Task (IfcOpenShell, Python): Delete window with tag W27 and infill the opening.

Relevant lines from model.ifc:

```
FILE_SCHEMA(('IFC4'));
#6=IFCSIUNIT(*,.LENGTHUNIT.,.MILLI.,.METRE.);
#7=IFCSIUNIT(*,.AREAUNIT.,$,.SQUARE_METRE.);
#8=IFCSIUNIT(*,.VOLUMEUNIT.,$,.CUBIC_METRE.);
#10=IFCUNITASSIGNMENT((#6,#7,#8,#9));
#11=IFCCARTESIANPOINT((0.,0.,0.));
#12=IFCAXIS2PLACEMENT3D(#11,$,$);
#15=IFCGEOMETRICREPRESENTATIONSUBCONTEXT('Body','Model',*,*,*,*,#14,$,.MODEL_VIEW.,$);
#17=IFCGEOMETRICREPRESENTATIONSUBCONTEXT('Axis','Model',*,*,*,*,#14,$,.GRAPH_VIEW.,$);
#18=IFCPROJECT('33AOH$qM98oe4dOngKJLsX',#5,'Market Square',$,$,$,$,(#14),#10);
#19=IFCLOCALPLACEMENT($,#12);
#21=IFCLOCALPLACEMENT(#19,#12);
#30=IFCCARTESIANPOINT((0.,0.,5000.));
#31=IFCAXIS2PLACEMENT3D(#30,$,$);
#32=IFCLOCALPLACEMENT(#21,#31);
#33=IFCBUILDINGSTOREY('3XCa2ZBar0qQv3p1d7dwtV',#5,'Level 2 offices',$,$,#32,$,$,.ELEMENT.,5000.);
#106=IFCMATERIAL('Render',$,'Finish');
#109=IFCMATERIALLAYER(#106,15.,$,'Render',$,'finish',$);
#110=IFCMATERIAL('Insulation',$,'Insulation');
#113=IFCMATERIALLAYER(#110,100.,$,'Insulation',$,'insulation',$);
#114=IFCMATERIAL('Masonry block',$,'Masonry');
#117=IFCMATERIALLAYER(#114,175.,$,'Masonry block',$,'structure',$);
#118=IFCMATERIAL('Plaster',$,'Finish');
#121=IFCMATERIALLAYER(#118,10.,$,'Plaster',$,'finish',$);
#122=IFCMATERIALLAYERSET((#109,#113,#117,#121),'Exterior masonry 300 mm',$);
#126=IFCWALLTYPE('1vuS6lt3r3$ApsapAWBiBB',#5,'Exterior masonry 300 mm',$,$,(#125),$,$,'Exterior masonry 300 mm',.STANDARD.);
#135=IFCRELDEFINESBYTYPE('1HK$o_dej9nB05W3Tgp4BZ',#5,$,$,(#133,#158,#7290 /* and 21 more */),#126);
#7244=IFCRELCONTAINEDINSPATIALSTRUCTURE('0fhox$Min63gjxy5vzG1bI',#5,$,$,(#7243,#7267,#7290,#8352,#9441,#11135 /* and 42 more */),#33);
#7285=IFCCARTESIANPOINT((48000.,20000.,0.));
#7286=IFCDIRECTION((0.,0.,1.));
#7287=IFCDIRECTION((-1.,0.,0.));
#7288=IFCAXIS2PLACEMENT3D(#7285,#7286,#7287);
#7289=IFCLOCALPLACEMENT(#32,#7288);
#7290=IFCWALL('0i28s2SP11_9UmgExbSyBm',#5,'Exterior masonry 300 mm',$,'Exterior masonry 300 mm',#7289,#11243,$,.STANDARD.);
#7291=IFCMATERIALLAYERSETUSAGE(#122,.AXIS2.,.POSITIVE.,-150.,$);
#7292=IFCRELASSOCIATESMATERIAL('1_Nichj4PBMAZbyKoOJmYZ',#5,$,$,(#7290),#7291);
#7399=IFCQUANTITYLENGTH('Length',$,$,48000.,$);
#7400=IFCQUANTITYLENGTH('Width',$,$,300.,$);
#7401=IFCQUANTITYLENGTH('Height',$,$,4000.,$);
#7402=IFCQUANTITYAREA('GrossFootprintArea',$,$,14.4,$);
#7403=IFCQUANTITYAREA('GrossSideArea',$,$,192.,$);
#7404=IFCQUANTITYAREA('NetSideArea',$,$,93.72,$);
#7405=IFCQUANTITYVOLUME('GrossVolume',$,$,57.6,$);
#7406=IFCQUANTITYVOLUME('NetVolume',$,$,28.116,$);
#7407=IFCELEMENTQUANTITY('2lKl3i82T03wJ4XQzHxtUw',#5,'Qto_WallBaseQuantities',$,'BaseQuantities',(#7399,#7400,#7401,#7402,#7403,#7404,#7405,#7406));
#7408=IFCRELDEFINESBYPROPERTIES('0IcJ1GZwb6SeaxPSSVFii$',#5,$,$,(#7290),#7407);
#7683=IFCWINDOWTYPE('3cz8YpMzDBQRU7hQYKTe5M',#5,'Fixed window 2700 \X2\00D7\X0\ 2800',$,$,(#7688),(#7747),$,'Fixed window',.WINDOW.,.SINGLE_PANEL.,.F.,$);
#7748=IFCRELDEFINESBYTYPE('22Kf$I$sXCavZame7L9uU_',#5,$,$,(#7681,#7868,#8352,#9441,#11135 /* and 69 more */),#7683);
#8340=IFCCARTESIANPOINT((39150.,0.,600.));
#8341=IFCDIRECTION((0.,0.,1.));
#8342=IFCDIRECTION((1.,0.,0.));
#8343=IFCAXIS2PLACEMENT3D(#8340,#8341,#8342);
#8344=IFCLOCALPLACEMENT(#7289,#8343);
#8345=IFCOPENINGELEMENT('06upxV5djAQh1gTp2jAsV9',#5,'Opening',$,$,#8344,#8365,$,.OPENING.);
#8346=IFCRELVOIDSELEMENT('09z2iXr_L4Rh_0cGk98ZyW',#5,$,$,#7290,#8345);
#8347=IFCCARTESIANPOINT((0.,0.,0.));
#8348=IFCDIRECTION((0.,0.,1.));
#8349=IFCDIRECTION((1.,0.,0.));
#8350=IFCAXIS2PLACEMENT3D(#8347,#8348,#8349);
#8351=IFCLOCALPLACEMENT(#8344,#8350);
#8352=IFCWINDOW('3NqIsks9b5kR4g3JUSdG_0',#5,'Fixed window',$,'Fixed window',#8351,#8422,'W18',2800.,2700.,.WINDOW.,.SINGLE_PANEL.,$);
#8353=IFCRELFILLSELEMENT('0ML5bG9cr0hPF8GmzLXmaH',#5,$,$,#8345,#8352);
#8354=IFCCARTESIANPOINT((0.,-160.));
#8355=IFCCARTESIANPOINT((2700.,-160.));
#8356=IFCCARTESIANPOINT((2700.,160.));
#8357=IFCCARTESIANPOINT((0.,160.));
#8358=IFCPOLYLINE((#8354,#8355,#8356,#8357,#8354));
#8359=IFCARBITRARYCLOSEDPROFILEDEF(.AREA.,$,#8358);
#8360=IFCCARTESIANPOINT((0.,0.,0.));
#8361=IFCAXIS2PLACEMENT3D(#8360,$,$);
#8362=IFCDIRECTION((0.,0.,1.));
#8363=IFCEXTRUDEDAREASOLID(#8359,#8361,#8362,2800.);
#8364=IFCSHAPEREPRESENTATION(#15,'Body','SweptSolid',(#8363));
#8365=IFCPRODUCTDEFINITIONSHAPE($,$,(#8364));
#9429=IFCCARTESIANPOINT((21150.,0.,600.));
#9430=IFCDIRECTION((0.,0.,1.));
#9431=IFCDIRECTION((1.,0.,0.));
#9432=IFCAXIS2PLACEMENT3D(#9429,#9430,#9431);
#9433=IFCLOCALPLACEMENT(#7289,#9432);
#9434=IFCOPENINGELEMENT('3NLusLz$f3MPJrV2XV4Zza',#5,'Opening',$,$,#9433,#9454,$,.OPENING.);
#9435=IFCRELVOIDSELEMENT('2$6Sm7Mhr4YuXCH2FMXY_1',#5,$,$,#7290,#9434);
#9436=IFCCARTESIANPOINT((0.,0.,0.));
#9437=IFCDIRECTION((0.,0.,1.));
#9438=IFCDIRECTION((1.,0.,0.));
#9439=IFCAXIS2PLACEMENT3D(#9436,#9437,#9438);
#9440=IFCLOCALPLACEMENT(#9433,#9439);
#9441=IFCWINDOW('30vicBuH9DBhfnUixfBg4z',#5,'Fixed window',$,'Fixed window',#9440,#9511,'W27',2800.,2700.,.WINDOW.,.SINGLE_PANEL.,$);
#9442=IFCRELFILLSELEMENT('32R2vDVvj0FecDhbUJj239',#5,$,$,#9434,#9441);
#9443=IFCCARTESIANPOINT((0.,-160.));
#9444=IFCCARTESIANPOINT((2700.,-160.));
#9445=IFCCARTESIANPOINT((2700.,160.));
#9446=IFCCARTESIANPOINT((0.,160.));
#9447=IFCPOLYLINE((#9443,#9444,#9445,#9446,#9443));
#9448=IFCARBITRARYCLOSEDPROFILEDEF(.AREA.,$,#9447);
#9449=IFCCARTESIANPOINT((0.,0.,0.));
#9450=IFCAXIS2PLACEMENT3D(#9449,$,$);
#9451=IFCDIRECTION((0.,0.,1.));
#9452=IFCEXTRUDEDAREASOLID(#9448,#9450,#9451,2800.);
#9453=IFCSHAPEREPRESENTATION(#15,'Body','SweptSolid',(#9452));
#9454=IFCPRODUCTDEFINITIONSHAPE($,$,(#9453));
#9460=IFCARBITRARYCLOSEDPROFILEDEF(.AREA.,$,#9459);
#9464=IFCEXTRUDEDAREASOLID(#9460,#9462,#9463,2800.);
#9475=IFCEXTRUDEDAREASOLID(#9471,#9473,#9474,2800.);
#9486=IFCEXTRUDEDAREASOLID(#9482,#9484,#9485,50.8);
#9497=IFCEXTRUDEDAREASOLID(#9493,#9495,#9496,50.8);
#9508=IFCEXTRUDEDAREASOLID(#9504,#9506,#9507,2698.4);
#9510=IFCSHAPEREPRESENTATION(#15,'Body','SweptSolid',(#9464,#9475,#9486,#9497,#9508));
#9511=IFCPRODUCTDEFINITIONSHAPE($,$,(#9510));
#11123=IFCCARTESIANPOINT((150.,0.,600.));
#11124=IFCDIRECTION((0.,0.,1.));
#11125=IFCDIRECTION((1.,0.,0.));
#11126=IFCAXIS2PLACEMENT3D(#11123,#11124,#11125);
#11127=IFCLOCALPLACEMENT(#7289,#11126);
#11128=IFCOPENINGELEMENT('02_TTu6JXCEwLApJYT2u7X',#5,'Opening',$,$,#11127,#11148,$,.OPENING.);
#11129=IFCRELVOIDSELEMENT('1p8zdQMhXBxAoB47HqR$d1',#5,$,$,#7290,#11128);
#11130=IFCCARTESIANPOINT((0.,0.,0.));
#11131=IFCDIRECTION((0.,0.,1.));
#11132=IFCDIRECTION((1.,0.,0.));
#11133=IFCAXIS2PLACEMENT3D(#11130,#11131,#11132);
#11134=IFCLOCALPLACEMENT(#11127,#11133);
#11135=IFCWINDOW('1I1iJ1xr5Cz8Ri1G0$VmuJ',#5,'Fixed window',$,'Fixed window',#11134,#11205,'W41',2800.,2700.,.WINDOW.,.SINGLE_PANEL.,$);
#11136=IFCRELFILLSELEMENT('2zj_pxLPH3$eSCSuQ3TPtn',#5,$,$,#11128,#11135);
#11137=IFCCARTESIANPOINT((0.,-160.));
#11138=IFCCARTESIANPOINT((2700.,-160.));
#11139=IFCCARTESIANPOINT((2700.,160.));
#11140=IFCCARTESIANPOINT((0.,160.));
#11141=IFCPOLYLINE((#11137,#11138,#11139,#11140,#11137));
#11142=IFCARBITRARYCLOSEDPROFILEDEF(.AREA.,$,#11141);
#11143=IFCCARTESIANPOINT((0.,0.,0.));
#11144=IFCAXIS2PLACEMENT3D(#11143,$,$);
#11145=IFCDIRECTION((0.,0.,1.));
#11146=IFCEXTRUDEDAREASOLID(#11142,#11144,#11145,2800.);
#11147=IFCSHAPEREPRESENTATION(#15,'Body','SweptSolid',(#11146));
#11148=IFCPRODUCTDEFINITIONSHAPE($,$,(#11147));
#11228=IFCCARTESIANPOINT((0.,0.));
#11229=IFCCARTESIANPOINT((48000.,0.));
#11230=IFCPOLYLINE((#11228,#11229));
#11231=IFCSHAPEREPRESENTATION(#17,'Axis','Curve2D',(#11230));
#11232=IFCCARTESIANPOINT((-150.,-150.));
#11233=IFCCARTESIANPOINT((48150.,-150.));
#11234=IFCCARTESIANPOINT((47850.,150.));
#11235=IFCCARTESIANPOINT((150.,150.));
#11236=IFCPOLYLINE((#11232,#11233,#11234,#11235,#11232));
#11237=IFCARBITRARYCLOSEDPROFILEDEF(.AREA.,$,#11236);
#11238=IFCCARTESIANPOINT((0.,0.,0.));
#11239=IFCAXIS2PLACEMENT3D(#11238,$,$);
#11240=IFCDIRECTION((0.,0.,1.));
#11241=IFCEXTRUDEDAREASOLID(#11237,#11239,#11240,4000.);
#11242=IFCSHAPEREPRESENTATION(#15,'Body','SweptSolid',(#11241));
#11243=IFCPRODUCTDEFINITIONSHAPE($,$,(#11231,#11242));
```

```python
import ifcopenshell
import ifcopenshell.api.feature
import ifcopenshell.api.pset
import ifcopenshell.api.root
import ifcopenshell.geom
import ifcopenshell.util.element
import ifcopenshell.util.shape
import ifcopenshell.util.unit

model = ifcopenshell.open("model.ifc")
area_scale = ifcopenshell.util.unit.calculate_unit_scale(model, "AREAUNIT")
volume_scale = ifcopenshell.util.unit.calculate_unit_scale(model, "VOLUMEUNIT")
settings = ifcopenshell.geom.settings()


def volume(element):
    """Net volume in cubic metres, openings subtracted."""
    shape = ifcopenshell.geom.create_shape(settings, element)
    return ifcopenshell.util.shape.get_volume(shape.geometry)


window = model.by_guid("30vicBuH9DBhfnUixfBg4z")
opening = window.FillsVoids[0].RelatingOpeningElement
wall = opening.VoidsElements[0].RelatingBuildingElement
before = volume(wall)

ifcopenshell.api.root.remove_product(model, product=window)
ifcopenshell.api.feature.remove_feature(model, feature=opening)

after = volume(wall)
thickness = 0.3  # wall thickness in metres

# Update the wall's stored quantities.
qto = model.by_id(ifcopenshell.util.element.get_pset(wall, "Qto_WallBaseQuantities", should_inherit=False)["id"])
ifcopenshell.api.pset.edit_qto(model, qto=qto, properties={
    "NetSideArea": after / thickness / area_scale,
    "NetVolume": after / volume_scale,
})

print(f"wall volume {before:.3f} -> {after:.3f} m3")

model.write("model_rev.ifc")
```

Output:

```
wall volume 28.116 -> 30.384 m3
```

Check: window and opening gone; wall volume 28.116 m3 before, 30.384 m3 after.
